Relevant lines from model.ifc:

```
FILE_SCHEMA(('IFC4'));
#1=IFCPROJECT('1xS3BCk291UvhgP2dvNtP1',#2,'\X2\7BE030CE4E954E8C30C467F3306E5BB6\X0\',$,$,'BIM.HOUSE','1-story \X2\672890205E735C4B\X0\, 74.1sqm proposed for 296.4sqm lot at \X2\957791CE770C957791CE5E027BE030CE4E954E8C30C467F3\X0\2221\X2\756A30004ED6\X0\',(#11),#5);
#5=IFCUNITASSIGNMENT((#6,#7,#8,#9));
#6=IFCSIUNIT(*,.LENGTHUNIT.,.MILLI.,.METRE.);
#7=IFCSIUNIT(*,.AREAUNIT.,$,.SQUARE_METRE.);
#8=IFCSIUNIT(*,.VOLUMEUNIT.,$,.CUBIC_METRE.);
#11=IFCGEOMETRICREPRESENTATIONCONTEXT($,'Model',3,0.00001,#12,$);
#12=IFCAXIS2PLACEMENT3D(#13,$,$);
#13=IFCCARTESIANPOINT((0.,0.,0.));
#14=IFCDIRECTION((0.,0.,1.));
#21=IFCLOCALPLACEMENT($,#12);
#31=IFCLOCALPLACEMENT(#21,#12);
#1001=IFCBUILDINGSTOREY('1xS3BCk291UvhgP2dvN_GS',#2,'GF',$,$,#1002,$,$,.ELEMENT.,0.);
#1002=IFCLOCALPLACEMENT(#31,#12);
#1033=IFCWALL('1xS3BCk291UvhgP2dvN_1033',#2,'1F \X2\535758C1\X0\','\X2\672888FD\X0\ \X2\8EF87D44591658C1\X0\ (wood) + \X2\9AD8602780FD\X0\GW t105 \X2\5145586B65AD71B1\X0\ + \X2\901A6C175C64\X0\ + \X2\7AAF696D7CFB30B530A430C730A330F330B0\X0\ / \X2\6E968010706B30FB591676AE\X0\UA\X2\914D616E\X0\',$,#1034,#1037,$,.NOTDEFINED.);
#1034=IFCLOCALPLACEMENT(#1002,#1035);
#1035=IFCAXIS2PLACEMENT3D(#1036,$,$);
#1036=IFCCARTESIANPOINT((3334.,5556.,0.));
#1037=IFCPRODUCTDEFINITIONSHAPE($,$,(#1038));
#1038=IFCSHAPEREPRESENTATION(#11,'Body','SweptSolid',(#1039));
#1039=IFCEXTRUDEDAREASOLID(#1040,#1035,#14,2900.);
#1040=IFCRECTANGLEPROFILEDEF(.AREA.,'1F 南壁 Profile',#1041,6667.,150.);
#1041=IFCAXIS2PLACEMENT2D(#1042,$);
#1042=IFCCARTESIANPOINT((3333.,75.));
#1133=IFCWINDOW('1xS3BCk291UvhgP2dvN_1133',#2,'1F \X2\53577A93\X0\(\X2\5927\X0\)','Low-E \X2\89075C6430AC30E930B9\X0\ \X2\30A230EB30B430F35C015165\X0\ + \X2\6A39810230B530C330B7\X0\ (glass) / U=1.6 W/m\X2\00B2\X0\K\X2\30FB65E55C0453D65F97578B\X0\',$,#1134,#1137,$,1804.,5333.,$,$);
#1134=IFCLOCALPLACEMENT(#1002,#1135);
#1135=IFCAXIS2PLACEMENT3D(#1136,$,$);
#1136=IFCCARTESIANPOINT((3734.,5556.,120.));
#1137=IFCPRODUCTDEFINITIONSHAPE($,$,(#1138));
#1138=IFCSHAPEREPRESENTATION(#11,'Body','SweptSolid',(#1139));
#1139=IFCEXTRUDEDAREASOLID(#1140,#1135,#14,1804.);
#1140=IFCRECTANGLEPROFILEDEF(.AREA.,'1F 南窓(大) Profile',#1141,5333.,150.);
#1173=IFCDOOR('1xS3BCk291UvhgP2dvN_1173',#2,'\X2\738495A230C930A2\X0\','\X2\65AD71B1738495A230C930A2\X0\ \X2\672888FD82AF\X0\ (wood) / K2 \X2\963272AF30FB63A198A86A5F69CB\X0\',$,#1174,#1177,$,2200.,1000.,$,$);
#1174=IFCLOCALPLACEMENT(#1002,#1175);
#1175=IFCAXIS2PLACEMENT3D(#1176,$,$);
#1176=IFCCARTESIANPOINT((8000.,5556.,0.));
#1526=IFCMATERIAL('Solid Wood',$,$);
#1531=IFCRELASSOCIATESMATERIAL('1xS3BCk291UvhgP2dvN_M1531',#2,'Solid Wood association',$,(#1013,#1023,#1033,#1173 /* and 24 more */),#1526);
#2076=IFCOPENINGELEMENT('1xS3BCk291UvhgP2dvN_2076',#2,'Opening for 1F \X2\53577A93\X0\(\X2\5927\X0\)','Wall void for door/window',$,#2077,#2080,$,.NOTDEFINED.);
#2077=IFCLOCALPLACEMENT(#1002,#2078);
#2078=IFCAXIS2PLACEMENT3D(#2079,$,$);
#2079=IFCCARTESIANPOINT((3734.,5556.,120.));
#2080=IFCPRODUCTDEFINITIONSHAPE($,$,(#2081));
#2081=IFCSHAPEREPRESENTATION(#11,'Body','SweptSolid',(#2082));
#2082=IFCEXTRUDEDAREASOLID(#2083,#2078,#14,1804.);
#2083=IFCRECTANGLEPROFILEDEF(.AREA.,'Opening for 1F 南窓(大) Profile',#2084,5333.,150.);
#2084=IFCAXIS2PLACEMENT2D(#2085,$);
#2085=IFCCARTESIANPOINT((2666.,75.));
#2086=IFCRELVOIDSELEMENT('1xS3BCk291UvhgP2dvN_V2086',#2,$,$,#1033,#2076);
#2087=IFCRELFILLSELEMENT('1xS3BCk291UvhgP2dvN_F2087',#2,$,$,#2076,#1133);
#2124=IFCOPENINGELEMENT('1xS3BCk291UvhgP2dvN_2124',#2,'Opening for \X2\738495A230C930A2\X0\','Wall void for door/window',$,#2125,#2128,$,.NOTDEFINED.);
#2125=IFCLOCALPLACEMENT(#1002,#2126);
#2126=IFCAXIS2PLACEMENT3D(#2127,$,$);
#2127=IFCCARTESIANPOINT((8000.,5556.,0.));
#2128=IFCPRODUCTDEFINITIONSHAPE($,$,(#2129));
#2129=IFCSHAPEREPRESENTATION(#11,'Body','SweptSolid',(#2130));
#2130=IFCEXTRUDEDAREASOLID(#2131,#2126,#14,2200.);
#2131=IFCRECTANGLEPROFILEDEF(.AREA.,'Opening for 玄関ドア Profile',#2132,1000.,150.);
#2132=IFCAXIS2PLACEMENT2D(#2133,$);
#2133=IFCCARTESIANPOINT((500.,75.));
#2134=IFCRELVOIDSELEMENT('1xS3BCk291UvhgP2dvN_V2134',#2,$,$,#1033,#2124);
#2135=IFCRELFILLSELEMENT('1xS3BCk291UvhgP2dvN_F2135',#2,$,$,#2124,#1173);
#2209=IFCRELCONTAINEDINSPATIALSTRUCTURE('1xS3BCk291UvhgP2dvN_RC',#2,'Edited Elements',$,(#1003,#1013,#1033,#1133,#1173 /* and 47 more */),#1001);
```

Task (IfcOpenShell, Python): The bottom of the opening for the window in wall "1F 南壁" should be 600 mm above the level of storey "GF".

```python
import numpy as np
import ifcopenshell
import ifcopenshell.api.geometry
import ifcopenshell.geom
import ifcopenshell.util.element
import ifcopenshell.util.placement
import ifcopenshell.util.shape
import ifcopenshell.util.unit

model = ifcopenshell.open("model.ifc")
unit_scale = ifcopenshell.util.unit.calculate_unit_scale(model)

window = model.by_guid("1xS3BCk291UvhgP2dvN_1133")
opening = window.FillsVoids[0].RelatingOpeningElement
storey = ifcopenshell.util.element.get_container(window, ifc_class="IfcBuildingStorey")
level = ifcopenshell.util.placement.get_local_placement(storey.ObjectPlacement)[2, 3]

# The opening's origin need not be at the sill, so measure its lowest point.
shape = ifcopenshell.geom.create_shape(ifcopenshell.geom.settings(), opening)
bottom = ifcopenshell.util.shape.get_shape_bottom_elevation(shape, shape.geometry) / unit_scale
dz = level + 0.6 / unit_scale - bottom

shift = np.array([0.0, 0.0, dz])
# The window is not placed relative to its opening, so move both.
for product in (opening, window):
    matrix = ifcopenshell.util.placement.get_local_placement(product.ObjectPlacement)
    matrix[:3, 3] += shift
    ifcopenshell.api.geometry.edit_object_placement(model, product=product, matrix=matrix, is_si=False)

print(f"moved by {dz * unit_scale:+.3f} m")

model.write("model_edited.ifc")
```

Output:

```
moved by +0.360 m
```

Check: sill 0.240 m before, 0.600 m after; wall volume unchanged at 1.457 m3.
